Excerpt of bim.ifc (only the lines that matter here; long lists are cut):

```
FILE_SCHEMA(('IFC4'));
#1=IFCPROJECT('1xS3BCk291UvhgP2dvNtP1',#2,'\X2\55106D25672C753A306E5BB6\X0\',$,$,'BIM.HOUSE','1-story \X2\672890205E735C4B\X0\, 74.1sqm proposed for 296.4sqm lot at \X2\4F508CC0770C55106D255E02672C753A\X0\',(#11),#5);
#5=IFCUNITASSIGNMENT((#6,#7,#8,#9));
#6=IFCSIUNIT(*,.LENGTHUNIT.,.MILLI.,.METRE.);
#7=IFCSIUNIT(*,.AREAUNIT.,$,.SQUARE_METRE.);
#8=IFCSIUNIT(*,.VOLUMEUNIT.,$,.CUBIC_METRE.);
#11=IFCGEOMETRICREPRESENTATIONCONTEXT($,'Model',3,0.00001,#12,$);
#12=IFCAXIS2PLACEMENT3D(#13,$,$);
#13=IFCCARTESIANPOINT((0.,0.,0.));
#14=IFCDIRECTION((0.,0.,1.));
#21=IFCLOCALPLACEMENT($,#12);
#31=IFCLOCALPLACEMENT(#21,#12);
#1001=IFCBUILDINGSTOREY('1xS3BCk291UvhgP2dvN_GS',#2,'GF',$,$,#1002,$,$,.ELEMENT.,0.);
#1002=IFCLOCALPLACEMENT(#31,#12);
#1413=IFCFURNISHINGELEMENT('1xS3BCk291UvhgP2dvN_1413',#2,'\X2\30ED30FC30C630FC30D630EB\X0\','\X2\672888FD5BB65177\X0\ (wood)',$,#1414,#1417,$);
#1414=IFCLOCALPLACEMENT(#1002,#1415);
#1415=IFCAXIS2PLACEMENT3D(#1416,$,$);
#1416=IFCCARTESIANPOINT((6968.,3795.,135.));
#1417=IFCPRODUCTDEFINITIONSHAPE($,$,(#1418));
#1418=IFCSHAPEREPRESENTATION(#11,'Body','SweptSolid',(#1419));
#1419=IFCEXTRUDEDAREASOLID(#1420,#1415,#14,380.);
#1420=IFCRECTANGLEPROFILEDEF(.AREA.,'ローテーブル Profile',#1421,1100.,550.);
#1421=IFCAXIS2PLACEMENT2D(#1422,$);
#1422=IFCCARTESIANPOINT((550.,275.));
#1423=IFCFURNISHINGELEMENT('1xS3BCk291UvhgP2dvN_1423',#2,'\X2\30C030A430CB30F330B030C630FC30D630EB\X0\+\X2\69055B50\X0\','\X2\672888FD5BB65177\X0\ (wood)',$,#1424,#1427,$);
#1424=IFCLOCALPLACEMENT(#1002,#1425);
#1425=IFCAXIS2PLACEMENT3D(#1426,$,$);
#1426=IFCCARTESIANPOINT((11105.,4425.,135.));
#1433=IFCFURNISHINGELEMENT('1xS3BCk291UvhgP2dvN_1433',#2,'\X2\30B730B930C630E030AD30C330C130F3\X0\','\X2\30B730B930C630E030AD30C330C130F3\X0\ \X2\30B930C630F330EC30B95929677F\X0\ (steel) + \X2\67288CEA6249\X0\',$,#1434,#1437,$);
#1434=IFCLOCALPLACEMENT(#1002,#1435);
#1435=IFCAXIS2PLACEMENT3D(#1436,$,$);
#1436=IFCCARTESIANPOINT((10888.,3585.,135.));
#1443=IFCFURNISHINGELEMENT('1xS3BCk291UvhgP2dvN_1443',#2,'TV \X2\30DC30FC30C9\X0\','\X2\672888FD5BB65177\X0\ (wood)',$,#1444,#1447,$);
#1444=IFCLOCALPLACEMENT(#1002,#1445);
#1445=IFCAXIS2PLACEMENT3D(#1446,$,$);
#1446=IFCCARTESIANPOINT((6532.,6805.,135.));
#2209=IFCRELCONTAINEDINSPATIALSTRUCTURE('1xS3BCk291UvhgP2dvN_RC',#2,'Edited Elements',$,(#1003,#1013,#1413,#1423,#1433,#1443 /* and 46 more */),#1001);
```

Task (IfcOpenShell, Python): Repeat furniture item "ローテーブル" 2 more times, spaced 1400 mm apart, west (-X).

```python
import numpy as np
import ifcopenshell
import ifcopenshell.api.geometry
import ifcopenshell.api.root
import ifcopenshell.util.element
import ifcopenshell.util.placement
import ifcopenshell.util.unit

model = ifcopenshell.open("bim.ifc")
unit_scale = ifcopenshell.util.unit.calculate_unit_scale(model)


def reuse_history(source, copy):
    """copy_class also copies each property set's owner history, people and application; keep the originals."""
    for rel in copy.IsDefinedBy:
        if rel.is_a("IfcRelDefinesByProperties") and (history := rel.RelatingPropertyDefinition.OwnerHistory):
            rel.RelatingPropertyDefinition.OwnerHistory = source.OwnerHistory
            ifcopenshell.util.element.remove_deep2(model, history)


source = model.by_guid("1xS3BCk291UvhgP2dvN_1413")
base = ifcopenshell.util.placement.get_local_placement(source.ObjectPlacement)
step = np.array([-1.0, 0.0, 0.0]) * 1.4 / unit_scale

for i in range(1, 3):
    copy = ifcopenshell.api.root.copy_class(model, product=source)
    copy.Representation = ifcopenshell.util.element.copy_deep(
        model, source.Representation, exclude=["IfcGeometricRepresentationContext", "IfcRepresentationMap"]
    )
    reuse_history(source, copy)
    matrix = base.copy()
    matrix[:3, 3] += i * step
    print("added at", matrix[:3, 3].round(3) + 0.0)
    ifcopenshell.api.geometry.edit_object_placement(model, product=copy, matrix=matrix, is_si=False)

model.write("bim_updated.ifc")
```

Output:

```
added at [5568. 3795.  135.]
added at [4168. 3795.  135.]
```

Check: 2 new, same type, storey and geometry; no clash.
